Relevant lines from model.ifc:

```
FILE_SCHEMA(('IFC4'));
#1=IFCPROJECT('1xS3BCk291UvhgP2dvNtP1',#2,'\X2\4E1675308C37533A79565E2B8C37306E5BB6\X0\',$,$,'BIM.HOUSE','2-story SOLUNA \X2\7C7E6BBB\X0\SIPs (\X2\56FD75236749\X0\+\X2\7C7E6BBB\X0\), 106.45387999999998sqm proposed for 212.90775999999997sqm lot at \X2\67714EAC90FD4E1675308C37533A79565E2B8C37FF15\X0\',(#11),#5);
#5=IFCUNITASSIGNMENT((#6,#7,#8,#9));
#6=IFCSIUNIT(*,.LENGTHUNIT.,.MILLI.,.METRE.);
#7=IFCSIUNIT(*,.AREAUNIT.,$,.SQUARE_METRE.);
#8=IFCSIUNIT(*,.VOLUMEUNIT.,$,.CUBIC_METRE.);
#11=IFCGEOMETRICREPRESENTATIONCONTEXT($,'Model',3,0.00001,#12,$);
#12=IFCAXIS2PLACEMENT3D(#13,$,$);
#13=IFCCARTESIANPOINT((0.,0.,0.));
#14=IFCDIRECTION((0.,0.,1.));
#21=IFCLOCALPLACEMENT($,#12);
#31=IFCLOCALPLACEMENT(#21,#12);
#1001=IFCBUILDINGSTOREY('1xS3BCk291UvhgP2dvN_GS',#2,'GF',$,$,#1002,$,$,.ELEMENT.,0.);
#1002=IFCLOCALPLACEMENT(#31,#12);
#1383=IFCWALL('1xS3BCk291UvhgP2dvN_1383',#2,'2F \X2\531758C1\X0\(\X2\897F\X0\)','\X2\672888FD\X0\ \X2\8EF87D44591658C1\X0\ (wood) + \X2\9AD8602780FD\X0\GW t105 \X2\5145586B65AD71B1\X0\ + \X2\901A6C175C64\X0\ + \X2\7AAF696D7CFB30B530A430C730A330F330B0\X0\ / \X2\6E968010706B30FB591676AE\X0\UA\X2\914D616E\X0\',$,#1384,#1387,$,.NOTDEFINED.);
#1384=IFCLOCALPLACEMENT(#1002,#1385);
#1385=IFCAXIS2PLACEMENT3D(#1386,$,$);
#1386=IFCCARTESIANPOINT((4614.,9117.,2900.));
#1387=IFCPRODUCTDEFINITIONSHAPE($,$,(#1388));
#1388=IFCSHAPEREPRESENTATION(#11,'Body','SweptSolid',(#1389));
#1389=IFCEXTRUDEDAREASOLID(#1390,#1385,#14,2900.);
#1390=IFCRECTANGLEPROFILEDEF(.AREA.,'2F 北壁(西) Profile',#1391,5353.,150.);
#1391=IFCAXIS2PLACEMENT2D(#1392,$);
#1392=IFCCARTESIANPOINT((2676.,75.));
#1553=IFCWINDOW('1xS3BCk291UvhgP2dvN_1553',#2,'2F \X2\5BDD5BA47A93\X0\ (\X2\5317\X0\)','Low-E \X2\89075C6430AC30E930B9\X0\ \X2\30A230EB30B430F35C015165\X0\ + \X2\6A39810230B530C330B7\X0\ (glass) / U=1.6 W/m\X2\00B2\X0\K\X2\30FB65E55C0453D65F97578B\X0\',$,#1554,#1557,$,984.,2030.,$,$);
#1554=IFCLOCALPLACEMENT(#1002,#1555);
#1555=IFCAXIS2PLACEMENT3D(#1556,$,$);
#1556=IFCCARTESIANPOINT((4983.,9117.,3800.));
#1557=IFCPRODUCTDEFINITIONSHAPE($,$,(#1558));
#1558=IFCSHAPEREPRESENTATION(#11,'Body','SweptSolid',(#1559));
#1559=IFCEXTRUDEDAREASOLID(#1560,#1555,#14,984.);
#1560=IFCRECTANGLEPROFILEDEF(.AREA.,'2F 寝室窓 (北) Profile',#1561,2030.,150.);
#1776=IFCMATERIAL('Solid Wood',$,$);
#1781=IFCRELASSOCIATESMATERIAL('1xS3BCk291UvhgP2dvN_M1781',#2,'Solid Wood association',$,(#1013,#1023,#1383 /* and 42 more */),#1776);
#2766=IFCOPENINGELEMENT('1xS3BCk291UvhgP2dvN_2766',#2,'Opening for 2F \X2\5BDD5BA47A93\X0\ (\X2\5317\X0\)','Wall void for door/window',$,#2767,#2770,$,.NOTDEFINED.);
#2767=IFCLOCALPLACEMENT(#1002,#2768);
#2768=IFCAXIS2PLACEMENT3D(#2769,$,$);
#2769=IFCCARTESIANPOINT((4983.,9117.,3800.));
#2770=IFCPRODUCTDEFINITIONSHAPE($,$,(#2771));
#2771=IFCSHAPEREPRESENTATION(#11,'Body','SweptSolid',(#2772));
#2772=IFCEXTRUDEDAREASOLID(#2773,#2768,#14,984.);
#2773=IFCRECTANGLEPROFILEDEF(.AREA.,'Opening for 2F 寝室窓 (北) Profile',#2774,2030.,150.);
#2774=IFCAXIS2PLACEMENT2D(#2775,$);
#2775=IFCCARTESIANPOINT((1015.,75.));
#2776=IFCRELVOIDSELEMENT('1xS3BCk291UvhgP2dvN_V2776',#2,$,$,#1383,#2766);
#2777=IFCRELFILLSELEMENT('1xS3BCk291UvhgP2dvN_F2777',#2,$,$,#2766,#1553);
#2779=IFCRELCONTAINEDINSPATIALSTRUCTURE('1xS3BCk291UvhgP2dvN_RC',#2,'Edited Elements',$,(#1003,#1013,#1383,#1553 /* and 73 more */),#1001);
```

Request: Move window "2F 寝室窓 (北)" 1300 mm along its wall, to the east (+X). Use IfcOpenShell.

```python
import ifcopenshell
import ifcopenshell.api.geometry
import ifcopenshell.util.placement
import ifcopenshell.util.unit

model = ifcopenshell.open("model.ifc")
unit_scale = ifcopenshell.util.unit.calculate_unit_scale(model)

window = model.by_id(1553)
opening = window.FillsVoids[0].RelatingOpeningElement
wall = opening.VoidsElements[0].RelatingBuildingElement

wall_matrix = ifcopenshell.util.placement.get_local_placement(wall.ObjectPlacement)
shift = wall_matrix[:3, 0] * 1.3 / unit_scale
before = ifcopenshell.util.placement.get_local_placement(window.ObjectPlacement)[:3, 3].copy()

# The window is not placed relative to its opening, so move both.
for product in (opening, window):
    matrix = ifcopenshell.util.placement.get_local_placement(product.ObjectPlacement)
    matrix[:3, 3] += shift
    ifcopenshell.api.geometry.edit_object_placement(model, product=product, matrix=matrix, is_si=False)

after = ifcopenshell.util.placement.get_local_placement(window.ObjectPlacement)[:3, 3]
print("window moved by", (after - before).round(3) + 0.0)

model.write("model_v2.ifc")
```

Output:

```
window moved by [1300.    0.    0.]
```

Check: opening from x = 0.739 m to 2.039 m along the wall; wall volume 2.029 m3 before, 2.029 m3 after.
